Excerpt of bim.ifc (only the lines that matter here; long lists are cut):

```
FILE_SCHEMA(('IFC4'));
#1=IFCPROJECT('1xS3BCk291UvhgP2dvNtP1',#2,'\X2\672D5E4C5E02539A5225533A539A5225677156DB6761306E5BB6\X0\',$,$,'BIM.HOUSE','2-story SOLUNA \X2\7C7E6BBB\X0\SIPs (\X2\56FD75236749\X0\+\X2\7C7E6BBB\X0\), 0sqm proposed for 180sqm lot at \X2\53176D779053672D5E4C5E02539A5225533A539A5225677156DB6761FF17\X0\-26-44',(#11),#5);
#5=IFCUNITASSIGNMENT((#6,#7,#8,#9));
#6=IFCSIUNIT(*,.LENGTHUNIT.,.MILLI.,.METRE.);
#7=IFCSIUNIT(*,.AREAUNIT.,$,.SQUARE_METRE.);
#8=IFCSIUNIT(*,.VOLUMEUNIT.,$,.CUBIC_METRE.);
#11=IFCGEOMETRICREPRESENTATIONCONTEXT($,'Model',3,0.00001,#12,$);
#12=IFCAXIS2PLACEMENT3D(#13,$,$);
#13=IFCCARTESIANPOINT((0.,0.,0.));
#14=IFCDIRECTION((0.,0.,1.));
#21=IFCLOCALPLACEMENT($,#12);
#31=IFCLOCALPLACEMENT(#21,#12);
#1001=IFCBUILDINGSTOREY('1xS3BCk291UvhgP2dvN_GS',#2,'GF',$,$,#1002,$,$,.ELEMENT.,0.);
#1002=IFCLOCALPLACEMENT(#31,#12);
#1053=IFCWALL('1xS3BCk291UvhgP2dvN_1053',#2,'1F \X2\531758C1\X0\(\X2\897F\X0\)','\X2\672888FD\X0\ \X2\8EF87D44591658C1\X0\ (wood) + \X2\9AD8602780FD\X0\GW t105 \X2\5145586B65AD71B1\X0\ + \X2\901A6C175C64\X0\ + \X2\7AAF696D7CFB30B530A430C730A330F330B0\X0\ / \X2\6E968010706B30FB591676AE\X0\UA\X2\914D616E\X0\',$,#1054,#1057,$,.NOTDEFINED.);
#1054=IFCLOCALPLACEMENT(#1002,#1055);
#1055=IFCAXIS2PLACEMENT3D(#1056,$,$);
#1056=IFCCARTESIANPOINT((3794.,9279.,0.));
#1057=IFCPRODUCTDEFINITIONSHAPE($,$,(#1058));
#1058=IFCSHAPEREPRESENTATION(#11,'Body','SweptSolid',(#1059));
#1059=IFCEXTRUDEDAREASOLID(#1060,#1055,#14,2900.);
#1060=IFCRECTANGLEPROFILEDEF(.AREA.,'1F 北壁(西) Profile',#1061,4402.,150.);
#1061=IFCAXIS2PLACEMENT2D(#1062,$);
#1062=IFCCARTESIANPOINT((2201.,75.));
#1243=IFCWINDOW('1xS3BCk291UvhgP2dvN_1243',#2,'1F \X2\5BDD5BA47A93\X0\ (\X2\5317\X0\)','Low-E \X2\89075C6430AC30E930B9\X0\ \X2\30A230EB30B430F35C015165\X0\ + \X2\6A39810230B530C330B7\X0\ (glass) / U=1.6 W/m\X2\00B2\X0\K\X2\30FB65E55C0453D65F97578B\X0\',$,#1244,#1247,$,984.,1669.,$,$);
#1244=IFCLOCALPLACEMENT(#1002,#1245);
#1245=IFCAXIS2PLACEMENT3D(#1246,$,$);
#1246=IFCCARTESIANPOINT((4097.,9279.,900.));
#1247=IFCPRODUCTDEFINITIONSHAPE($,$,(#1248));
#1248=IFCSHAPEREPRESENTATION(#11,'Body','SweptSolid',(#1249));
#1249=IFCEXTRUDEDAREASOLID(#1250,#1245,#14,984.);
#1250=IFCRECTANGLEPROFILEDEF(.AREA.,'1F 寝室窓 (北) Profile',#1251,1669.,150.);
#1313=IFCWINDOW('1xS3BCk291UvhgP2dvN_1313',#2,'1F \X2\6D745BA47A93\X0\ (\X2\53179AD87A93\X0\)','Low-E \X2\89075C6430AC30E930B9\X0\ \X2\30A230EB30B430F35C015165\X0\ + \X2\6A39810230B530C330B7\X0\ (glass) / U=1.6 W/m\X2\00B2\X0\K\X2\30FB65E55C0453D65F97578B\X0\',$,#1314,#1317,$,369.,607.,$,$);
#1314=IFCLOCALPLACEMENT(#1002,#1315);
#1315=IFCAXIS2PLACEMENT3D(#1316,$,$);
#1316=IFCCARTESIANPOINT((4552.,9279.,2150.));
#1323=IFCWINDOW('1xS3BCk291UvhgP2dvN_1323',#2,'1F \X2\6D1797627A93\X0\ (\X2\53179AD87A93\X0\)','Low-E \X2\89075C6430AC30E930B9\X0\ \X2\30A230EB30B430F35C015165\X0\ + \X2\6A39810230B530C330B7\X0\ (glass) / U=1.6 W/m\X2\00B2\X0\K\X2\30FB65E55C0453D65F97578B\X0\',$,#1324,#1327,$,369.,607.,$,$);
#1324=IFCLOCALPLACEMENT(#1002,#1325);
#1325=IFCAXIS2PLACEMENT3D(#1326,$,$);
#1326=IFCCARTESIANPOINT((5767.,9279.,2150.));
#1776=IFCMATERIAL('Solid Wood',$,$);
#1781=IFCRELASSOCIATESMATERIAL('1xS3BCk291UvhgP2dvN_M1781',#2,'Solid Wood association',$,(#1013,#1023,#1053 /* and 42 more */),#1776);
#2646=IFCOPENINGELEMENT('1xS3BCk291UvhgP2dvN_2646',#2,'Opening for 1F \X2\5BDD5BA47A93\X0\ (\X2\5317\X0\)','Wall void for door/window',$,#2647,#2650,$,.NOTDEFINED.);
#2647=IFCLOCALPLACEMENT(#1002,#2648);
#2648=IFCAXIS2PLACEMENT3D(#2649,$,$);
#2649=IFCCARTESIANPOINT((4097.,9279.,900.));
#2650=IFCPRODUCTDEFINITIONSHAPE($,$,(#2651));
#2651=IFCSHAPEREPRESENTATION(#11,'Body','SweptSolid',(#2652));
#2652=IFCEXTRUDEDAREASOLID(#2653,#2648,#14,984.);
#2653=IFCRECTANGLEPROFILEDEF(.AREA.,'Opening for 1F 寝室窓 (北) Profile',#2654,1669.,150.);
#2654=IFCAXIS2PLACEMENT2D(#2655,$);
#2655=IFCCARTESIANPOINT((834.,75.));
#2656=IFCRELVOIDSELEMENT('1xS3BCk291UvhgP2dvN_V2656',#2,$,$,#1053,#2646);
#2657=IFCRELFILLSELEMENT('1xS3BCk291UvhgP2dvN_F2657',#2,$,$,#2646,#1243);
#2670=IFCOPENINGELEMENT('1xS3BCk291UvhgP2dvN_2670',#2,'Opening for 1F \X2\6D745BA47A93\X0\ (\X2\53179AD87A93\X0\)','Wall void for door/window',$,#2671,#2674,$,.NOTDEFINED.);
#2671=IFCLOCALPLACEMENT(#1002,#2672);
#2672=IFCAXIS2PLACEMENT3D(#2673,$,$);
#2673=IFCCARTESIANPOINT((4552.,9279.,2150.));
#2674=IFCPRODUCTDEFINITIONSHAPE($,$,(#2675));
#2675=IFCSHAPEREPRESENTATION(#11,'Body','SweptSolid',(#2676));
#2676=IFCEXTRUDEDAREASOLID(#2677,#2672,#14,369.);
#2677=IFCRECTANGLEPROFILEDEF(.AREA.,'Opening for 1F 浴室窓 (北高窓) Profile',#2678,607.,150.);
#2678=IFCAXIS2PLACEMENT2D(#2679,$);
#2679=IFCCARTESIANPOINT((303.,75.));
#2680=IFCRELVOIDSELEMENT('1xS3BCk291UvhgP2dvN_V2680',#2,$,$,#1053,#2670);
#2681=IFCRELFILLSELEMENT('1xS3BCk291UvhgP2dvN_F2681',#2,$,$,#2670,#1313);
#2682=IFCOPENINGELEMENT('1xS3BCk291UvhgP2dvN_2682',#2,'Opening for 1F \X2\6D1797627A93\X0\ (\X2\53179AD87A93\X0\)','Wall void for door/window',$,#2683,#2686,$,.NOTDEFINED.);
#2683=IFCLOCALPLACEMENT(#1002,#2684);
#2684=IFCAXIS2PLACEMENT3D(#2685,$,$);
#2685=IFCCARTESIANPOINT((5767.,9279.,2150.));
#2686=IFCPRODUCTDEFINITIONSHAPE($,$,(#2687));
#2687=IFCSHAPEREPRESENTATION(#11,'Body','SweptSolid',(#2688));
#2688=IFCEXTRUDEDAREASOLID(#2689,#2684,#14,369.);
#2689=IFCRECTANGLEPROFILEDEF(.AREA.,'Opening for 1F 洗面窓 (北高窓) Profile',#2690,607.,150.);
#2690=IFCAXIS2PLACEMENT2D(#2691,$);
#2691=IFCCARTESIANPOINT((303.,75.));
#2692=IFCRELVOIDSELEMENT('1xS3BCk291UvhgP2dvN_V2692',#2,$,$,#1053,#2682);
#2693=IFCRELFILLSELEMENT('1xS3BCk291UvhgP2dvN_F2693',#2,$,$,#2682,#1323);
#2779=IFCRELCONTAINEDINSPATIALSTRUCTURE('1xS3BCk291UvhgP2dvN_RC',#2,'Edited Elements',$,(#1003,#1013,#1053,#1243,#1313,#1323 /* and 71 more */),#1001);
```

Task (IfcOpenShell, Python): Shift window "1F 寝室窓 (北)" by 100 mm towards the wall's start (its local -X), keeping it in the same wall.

```python
import ifcopenshell
import ifcopenshell.api.geometry
import ifcopenshell.util.placement
import ifcopenshell.util.unit

model = ifcopenshell.open("bim.ifc")
unit_scale = ifcopenshell.util.unit.calculate_unit_scale(model)

window = model.by_id(1243)
opening = window.FillsVoids[0].RelatingOpeningElement
wall = opening.VoidsElements[0].RelatingBuildingElement

wall_matrix = ifcopenshell.util.placement.get_local_placement(wall.ObjectPlacement)
shift = wall_matrix[:3, 0] * -0.1 / unit_scale
before = ifcopenshell.util.placement.get_local_placement(window.ObjectPlacement)[:3, 3].copy()

# The window is not placed relative to its opening, so move both.
for product in (opening, window):
    matrix = ifcopenshell.util.placement.get_local_placement(product.ObjectPlacement)
    matrix[:3, 3] += shift
    ifcopenshell.api.geometry.edit_object_placement(model, product=product, matrix=matrix, is_si=False)

after = ifcopenshell.util.placement.get_local_placement(window.ObjectPlacement)[:3, 3]
print("window moved by", (after - before).round(3) + 0.0)

model.write("bim-out.ifc")
```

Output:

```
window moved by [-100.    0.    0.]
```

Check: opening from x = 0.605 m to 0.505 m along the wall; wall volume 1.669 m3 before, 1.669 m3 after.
